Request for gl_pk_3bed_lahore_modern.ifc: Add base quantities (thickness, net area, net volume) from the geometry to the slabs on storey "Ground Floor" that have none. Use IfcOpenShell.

First a look at what the model holds.

```python
import ifcopenshell
import ifcopenshell.util.element
import ifcopenshell.util.unit

model = ifcopenshell.open("gl_pk_3bed_lahore_modern.ifc")
print(model.schema)
for unit_type in ("LENGTHUNIT", "AREAUNIT", "VOLUMEUNIT"):
    print(unit_type, ifcopenshell.util.unit.calculate_unit_scale(model, unit_type))
storey = next(s for s in model.by_type("IfcBuildingStorey") if s.Name == "Ground Floor")
slabs = [e for e in ifcopenshell.util.element.get_decomposition(storey) if e.is_a("IfcSlab")]
for e in sorted(slabs, key=lambda e: e.id()):
    print(e.id(), e.is_a(), e.Name, list(ifcopenshell.util.element.get_psets(e, qtos_only=True)), sep=" | ")
```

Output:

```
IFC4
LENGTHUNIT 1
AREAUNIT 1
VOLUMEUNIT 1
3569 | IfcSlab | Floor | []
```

```python
import ifcopenshell
import ifcopenshell.api.pset
import ifcopenshell.geom
import ifcopenshell.util.element
import ifcopenshell.util.shape
import ifcopenshell.util.unit

model = ifcopenshell.open("gl_pk_3bed_lahore_modern.ifc")
unit_scale = ifcopenshell.util.unit.calculate_unit_scale(model)
area_scale = ifcopenshell.util.unit.calculate_unit_scale(model, "AREAUNIT")
volume_scale = ifcopenshell.util.unit.calculate_unit_scale(model, "VOLUMEUNIT")
settings = ifcopenshell.geom.settings()

storey = next(s for s in model.by_type("IfcBuildingStorey") if s.Name == "Ground Floor")
slabs = [e for e in ifcopenshell.util.element.get_decomposition(storey) if e.is_a("IfcSlab")]

for e in sorted(slabs, key=lambda e: e.id()):
    if ifcopenshell.util.element.get_psets(e, qtos_only=True, should_inherit=False):
        continue
    # Geometry comes back in metres, in the element's own axes.
    shape = ifcopenshell.geom.create_shape(settings, e)
    values = {
        "Width": ifcopenshell.util.shape.get_z(shape.geometry) / unit_scale,
        "NetArea": ifcopenshell.util.shape.get_footprint_area(shape.geometry) / area_scale,
        "NetVolume": ifcopenshell.util.shape.get_volume(shape.geometry) / volume_scale,
    }
    qto = ifcopenshell.api.pset.add_qto(model, product=e, name="Qto_SlabBaseQuantities")
    ifcopenshell.api.pset.edit_qto(model, qto=qto, properties=values)
    print(e.id(), {k: round(v, 3) for k, v in values.items()})

model.write("gl_pk_3bed_lahore_modern_v2.ifc")
```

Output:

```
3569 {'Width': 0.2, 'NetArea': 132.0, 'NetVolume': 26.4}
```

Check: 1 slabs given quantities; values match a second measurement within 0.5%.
